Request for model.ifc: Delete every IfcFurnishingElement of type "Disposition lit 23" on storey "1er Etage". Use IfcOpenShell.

First a look at what the model holds.

```python
import ifcopenshell
import ifcopenshell.util.element

model = ifcopenshell.open("model.ifc")
print(model.schema)
storey = next(s for s in model.by_type("IfcBuildingStorey") if s.Name == "1er Etage")
furniture = [e for e in ifcopenshell.util.element.get_decomposition(storey) if e.is_a("IfcFurnishingElement")]
seen = {}
for e in furniture:
    element_type = ifcopenshell.util.element.get_type(e)
    name = element_type.Name if element_type not in (None, e) else None
    seen[name] = seen.get(name, 0) + 1
for name, count in sorted(seen.items(), key=str):
    print(count, "x", name)
```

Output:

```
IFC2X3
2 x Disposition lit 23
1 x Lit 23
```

```python
import ifcopenshell
import ifcopenshell.api.root
import ifcopenshell.util.element

model = ifcopenshell.open("model.ifc")

storey = next(s for s in model.by_type("IfcBuildingStorey") if s.Name == "1er Etage")
furniture = [e for e in ifcopenshell.util.element.get_decomposition(storey) if e.is_a("IfcFurnishingElement")]
targets = [e for e in furniture if (t := ifcopenshell.util.element.get_type(e)) not in (None, e) and t.Name == "Disposition lit 23"]

for e in targets:
    ifcopenshell.api.root.remove_product(model, product=e)
print(len(targets), "removed")

model.write("model_rev.ifc")
```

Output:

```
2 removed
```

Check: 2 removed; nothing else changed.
